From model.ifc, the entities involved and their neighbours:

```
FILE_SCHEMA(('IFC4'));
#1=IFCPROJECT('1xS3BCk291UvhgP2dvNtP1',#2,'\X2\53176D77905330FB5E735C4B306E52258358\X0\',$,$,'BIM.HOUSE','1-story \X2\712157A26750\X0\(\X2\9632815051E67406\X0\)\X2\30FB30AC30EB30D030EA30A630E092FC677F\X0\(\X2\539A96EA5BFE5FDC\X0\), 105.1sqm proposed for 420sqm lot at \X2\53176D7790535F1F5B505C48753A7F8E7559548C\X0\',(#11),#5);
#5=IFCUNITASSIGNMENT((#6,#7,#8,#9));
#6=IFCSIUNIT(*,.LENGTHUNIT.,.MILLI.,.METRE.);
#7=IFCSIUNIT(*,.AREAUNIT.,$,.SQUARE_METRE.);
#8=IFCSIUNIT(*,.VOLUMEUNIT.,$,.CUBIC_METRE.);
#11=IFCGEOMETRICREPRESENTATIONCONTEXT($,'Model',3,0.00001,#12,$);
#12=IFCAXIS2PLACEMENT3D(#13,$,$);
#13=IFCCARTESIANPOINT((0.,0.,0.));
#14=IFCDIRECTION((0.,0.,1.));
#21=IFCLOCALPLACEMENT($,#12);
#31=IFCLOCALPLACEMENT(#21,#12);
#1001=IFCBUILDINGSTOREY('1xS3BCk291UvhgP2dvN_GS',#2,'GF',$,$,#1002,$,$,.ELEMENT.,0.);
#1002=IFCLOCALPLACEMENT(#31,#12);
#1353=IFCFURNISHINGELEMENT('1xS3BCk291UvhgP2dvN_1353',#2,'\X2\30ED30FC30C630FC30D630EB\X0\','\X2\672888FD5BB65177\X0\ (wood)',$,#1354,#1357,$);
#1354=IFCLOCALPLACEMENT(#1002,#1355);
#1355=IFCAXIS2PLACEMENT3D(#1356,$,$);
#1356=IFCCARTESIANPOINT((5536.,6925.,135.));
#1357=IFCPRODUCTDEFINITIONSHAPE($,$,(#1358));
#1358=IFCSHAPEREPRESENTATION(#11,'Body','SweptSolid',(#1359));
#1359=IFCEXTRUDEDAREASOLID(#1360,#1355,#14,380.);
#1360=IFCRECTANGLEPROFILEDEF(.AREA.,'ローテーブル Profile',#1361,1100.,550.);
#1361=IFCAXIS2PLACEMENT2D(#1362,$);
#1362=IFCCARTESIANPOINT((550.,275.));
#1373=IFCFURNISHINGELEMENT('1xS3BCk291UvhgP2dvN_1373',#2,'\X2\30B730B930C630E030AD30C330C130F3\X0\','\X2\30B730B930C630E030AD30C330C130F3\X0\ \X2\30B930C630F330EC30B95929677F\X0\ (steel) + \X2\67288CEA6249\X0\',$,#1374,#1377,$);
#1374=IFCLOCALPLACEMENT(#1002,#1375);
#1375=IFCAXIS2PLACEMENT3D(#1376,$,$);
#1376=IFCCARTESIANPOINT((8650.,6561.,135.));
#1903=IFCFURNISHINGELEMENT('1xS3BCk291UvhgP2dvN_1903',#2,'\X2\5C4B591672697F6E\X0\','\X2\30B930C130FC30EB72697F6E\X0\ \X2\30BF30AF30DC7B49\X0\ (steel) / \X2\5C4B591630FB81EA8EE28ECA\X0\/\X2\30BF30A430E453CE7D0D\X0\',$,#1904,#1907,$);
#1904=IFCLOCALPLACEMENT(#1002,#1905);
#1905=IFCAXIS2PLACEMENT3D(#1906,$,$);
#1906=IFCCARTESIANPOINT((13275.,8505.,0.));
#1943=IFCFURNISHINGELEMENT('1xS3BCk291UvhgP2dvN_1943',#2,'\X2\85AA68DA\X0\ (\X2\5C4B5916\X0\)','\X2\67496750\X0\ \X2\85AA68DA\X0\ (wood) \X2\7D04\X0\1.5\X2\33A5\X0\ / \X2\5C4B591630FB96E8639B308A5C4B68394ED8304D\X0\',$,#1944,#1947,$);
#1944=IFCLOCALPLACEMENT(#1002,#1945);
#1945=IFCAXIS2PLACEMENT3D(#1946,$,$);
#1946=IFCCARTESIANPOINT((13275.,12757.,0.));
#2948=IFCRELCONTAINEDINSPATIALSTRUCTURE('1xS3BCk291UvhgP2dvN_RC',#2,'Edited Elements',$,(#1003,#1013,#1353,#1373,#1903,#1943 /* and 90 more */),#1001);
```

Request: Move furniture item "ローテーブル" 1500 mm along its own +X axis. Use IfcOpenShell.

```python
import ifcopenshell
import ifcopenshell.api.geometry
import ifcopenshell.util.placement
import ifcopenshell.util.unit

model = ifcopenshell.open("model.ifc")
unit_scale = ifcopenshell.util.unit.calculate_unit_scale(model)

item = model.by_guid("1xS3BCk291UvhgP2dvN_1353")
matrix = ifcopenshell.util.placement.get_local_placement(item.ObjectPlacement)
matrix[:3, 3] += matrix[:3, 0] * 1.5 / unit_scale
ifcopenshell.api.geometry.edit_object_placement(model, product=item, matrix=matrix, is_si=False)

print(ifcopenshell.util.placement.get_local_placement(item.ObjectPlacement).round(3) + 0.0)

model.write("model_updated.ifc")
```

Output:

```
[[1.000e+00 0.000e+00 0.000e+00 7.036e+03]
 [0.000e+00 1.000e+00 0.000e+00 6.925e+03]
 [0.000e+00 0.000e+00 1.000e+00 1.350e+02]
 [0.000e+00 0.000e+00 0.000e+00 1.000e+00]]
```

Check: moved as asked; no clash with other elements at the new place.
